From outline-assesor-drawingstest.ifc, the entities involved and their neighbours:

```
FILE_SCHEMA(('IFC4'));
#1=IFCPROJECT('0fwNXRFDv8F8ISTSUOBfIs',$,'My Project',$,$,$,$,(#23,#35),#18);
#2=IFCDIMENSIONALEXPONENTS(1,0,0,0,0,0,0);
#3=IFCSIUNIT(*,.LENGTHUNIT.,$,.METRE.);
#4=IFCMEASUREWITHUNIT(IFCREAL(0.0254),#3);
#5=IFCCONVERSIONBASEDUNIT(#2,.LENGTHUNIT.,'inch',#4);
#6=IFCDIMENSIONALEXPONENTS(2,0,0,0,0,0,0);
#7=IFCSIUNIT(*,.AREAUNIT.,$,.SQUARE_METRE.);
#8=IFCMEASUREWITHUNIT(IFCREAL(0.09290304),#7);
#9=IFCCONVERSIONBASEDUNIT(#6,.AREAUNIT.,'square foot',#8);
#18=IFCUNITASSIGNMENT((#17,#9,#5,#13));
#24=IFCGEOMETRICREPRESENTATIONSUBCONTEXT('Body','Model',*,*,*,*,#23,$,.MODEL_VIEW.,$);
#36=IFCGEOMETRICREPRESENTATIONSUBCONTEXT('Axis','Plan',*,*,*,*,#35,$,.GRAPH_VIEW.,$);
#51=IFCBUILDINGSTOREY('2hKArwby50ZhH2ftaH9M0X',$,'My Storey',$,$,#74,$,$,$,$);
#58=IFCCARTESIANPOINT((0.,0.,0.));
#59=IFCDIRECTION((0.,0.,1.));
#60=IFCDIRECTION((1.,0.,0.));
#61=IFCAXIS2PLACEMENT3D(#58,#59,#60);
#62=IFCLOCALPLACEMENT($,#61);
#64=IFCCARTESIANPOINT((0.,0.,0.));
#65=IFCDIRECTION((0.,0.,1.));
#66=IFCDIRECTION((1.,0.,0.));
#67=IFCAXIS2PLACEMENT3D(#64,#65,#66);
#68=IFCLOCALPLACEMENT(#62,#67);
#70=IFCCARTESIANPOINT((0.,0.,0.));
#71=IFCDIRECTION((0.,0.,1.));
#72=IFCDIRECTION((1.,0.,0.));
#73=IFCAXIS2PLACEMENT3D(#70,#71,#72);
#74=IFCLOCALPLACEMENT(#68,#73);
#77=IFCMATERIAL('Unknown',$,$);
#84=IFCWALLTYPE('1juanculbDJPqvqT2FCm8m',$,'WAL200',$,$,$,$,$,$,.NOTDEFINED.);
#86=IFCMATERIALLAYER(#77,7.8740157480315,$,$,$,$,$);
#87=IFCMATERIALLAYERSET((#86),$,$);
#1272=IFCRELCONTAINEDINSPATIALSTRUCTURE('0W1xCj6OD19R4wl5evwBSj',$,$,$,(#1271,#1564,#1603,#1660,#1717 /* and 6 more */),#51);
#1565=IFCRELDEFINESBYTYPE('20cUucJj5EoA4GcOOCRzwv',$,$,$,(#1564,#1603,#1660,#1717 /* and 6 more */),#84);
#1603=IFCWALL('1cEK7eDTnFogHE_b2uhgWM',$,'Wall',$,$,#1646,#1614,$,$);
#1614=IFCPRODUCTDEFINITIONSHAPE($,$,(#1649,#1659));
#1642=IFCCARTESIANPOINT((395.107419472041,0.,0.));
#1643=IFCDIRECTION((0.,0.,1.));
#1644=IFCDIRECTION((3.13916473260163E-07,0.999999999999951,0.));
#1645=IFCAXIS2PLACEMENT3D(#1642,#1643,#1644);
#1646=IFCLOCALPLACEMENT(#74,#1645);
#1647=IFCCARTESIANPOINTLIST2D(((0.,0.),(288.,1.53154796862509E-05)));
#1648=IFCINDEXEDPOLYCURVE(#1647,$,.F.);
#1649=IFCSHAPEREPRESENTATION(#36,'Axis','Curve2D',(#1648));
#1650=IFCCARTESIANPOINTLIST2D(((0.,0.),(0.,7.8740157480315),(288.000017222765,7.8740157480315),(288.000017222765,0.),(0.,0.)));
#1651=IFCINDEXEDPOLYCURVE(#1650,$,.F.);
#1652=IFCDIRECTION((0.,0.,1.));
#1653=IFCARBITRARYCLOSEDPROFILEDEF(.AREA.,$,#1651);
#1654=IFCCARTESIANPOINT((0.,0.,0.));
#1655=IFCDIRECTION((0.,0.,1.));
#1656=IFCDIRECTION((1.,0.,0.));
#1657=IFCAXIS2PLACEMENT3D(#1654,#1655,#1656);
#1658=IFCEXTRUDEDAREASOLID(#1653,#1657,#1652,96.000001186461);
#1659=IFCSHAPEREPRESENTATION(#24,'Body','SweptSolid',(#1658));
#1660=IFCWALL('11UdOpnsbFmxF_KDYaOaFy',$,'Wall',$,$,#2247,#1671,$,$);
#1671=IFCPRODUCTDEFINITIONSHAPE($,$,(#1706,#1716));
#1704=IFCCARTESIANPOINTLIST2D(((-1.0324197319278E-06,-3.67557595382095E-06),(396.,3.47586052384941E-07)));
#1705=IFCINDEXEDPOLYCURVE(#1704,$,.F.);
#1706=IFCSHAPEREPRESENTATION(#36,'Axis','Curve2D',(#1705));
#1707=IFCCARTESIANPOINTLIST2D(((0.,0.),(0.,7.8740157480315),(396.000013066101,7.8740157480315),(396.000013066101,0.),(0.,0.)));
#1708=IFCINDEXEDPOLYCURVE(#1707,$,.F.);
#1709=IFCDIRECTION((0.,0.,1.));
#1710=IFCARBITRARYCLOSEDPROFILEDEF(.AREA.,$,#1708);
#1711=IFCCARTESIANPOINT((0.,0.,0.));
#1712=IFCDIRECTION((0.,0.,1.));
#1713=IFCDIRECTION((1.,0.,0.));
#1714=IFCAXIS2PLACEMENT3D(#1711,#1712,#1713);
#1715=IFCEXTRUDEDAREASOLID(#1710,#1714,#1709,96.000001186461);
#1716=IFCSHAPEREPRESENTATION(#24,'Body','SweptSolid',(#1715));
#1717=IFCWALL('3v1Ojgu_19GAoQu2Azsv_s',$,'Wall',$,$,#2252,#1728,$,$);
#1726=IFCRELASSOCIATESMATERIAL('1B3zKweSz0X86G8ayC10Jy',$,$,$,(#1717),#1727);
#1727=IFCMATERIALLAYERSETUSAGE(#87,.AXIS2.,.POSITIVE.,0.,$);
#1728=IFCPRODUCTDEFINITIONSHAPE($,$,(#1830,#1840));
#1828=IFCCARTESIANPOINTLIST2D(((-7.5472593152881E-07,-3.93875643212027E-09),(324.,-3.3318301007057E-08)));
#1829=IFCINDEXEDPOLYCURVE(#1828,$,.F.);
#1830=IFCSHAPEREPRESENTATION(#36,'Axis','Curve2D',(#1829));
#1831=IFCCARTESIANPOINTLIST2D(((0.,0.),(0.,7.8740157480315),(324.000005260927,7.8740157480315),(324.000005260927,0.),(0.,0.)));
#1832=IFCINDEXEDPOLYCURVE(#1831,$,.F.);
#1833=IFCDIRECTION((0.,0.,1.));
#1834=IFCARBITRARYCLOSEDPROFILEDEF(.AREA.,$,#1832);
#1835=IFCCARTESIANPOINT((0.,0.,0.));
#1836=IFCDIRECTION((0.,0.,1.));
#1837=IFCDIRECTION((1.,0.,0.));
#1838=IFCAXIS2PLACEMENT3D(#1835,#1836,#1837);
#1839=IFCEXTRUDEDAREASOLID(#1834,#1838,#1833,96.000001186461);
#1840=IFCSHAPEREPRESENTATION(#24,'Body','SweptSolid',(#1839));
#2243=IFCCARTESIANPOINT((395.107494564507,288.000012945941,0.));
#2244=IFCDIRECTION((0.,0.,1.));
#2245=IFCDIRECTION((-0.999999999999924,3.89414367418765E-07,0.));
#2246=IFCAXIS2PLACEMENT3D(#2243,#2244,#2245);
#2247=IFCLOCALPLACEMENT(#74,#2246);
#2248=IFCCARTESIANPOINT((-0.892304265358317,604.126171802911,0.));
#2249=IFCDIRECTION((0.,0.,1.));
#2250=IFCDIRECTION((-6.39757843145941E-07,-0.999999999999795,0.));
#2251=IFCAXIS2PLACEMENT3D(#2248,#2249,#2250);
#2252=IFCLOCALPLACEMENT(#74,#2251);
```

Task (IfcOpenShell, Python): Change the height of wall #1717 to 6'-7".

```python
import ifcopenshell
import ifcopenshell.geom
import ifcopenshell.util.representation
import ifcopenshell.util.shape
import ifcopenshell.util.unit

model = ifcopenshell.open("outline-assesor-drawingstest.ifc")
unit_scale = ifcopenshell.util.unit.calculate_unit_scale(model)
settings = ifcopenshell.geom.settings()


def volume(element):
    """Net volume in cubic metres, openings subtracted."""
    shape = ifcopenshell.geom.create_shape(settings, element)
    return ifcopenshell.util.shape.get_volume(shape.geometry)


wall = model.by_guid("3v1Ojgu_19GAoQu2Azsv_s")
before = volume(wall)

body = ifcopenshell.util.representation.get_representation(wall, "Model", "Body")
solid = body.Items[0]
old_height = solid.Depth
solid.Depth = 79 * 0.0254 / unit_scale
after = volume(wall)

print(f"height {old_height:g} -> {solid.Depth:g}, volume {before:.3f} -> {after:.3f} m3")

model.write("outline-assesor-drawingstest-out.ifc")
```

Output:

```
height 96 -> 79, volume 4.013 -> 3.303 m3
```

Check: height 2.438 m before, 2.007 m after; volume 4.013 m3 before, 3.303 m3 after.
